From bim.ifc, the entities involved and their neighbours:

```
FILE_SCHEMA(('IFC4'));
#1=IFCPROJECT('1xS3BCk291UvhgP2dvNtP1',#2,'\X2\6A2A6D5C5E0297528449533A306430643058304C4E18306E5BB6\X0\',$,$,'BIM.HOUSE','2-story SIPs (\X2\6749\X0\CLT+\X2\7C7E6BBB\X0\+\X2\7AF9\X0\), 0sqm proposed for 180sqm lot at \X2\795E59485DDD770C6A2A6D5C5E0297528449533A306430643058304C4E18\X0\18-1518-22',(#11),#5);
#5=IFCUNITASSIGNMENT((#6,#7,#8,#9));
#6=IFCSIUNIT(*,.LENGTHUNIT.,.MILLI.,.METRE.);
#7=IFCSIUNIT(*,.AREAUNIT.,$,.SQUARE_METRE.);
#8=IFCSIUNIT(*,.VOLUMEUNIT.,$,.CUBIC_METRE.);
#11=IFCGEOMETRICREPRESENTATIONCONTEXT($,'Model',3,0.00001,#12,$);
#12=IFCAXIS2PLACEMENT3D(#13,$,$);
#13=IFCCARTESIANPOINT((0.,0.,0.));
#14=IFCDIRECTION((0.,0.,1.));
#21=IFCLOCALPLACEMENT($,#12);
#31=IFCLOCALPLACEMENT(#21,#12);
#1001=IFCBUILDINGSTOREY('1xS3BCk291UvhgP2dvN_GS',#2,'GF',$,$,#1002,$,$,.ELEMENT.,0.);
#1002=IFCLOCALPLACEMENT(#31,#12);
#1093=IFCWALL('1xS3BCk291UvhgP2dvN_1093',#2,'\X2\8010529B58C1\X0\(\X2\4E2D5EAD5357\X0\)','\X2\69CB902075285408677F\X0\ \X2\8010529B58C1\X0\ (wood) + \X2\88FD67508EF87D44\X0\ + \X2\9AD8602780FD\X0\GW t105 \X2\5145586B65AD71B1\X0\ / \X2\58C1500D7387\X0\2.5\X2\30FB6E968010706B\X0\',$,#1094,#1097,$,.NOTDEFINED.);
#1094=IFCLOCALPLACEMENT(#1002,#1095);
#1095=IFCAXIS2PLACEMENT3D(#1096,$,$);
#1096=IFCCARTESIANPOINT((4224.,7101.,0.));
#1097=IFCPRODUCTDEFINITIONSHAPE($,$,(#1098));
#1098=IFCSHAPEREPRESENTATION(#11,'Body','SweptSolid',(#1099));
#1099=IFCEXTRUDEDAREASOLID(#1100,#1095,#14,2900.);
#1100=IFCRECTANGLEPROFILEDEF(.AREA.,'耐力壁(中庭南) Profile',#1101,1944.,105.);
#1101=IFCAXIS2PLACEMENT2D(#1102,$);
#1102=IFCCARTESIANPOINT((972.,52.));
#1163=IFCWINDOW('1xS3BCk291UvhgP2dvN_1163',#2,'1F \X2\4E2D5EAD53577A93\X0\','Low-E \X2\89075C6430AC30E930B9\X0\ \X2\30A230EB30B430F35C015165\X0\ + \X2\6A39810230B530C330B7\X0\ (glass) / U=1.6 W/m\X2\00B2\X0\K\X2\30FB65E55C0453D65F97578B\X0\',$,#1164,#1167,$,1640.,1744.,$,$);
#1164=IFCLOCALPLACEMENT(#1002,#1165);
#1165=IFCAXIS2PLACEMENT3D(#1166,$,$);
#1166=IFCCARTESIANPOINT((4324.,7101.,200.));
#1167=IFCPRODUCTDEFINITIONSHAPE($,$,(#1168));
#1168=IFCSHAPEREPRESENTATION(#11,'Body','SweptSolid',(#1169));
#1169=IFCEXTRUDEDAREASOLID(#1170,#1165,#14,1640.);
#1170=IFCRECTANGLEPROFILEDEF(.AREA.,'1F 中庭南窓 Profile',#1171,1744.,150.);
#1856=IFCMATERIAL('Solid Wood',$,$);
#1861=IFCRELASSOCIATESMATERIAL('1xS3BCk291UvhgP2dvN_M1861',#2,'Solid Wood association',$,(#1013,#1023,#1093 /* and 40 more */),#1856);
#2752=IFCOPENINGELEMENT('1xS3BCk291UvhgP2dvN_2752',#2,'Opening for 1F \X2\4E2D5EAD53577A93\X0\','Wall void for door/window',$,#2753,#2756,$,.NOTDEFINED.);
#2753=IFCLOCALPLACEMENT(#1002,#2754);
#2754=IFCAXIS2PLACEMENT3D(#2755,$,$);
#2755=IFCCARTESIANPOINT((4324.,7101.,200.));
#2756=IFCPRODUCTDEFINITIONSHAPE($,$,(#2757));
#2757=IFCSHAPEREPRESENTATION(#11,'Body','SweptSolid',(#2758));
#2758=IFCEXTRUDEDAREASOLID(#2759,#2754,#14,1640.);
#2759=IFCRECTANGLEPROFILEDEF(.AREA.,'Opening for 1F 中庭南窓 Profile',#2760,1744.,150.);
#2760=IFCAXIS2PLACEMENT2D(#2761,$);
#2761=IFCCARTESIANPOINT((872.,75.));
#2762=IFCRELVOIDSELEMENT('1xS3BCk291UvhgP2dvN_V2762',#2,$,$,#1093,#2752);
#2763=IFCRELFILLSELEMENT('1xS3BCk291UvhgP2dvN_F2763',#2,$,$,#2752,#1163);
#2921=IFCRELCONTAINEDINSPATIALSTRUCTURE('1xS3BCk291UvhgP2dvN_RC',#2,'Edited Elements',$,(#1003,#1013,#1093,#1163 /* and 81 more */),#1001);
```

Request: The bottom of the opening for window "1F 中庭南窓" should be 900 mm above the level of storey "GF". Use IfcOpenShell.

```python
import numpy as np
import ifcopenshell
import ifcopenshell.api.geometry
import ifcopenshell.geom
import ifcopenshell.util.element
import ifcopenshell.util.placement
import ifcopenshell.util.shape
import ifcopenshell.util.unit

model = ifcopenshell.open("bim.ifc")
unit_scale = ifcopenshell.util.unit.calculate_unit_scale(model)

window = model.by_guid("1xS3BCk291UvhgP2dvN_1163")
opening = window.FillsVoids[0].RelatingOpeningElement
storey = ifcopenshell.util.element.get_container(window, ifc_class="IfcBuildingStorey")
level = ifcopenshell.util.placement.get_local_placement(storey.ObjectPlacement)[2, 3]

# The opening's origin need not be at the sill, so measure its lowest point.
shape = ifcopenshell.geom.create_shape(ifcopenshell.geom.settings(), opening)
bottom = ifcopenshell.util.shape.get_shape_bottom_elevation(shape, shape.geometry) / unit_scale
dz = level + 0.9 / unit_scale - bottom

shift = np.array([0.0, 0.0, dz])
# The window is not placed relative to its opening, so move both.
for product in (opening, window):
    matrix = ifcopenshell.util.placement.get_local_placement(product.ObjectPlacement)
    matrix[:3, 3] += shift
    ifcopenshell.api.geometry.edit_object_placement(model, product=product, matrix=matrix, is_si=False)

print(f"moved by {dz * unit_scale:+.3f} m")

model.write("bim_v2.ifc")
```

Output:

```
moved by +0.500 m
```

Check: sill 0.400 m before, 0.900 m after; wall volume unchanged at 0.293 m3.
